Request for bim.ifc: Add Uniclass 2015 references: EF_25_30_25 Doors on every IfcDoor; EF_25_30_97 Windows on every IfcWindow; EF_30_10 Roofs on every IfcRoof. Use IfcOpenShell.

First a look at what the model holds.

```python
import ifcopenshell

model = ifcopenshell.open("bim.ifc")
print(model.schema)
print("classifications:", [c.Name for c in model.by_type("IfcClassification")])
for ifc_class in ("IfcDoor", "IfcRoof", "IfcStair", "IfcWall", "IfcWindow"):
    print(ifc_class, len(model.by_type(ifc_class)))
```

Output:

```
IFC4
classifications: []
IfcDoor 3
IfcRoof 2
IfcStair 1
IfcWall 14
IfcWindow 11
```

```python
import ifcopenshell
import ifcopenshell.api.classification

model = ifcopenshell.open("bim.ifc")

system = ifcopenshell.api.classification.add_classification(model, classification="Uniclass 2015")

codes = {
    "IfcDoor": ("EF_25_30_25", "Doors"),
    "IfcWindow": ("EF_25_30_97", "Windows"),
    "IfcRoof": ("EF_30_10", "Roofs"),
}
for ifc_class, (code, name) in codes.items():
    products = model.by_type(ifc_class)
    ifcopenshell.api.classification.add_reference(
        model, products=products, classification=system, identification=code, name=name
    )
    print(code, len(products))

model.write("bim_updated.ifc")
```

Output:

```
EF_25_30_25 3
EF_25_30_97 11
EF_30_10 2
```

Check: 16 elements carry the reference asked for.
